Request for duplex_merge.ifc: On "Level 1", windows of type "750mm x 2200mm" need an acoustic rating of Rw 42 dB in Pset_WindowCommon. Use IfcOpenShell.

First a look at what the model holds.

```python
import ifcopenshell
import ifcopenshell.util.element

model = ifcopenshell.open("duplex_merge.ifc")
print(model.schema)
storey = next(s for s in model.by_type("IfcBuildingStorey") if s.Name == "Level 1")
windows = [e for e in ifcopenshell.util.element.get_decomposition(storey) if e.is_a("IfcWindow")]
seen = {}
for e in windows:
    element_type = ifcopenshell.util.element.get_type(e)
    key = (element_type.Name if element_type != e and element_type else None, ifcopenshell.util.element.get_pset(e, "Pset_WindowCommon", "AcousticRating"))
    seen[key] = seen.get(key, 0) + 1
for (name, value), count in sorted(seen.items(), key=str):
    print(count, "x", name, "|", value)
```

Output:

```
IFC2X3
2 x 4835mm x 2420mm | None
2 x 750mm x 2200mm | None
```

```python
import ifcopenshell
import ifcopenshell.api.pset
import ifcopenshell.util.element

model = ifcopenshell.open("duplex_merge.ifc")

storey = next(s for s in model.by_type("IfcBuildingStorey") if s.Name == "Level 1")
windows = [e for e in ifcopenshell.util.element.get_decomposition(storey) if e.is_a("IfcWindow")]

count = 0
for e in windows:
    element_type = ifcopenshell.util.element.get_type(e)
    if element_type in (None, e) or element_type.Name != "750mm x 2200mm":
        continue
    # add_pset returns the element's existing set when there is one.
    pset = ifcopenshell.api.pset.add_pset(model, product=e, name="Pset_WindowCommon")
    ifcopenshell.api.pset.edit_pset(model, pset=pset, properties={"AcousticRating": "Rw 42 dB"})
    count += 1

print(count, "windows updated")

model.write("duplex_merge-out.ifc")
```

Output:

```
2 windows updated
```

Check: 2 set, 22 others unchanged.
